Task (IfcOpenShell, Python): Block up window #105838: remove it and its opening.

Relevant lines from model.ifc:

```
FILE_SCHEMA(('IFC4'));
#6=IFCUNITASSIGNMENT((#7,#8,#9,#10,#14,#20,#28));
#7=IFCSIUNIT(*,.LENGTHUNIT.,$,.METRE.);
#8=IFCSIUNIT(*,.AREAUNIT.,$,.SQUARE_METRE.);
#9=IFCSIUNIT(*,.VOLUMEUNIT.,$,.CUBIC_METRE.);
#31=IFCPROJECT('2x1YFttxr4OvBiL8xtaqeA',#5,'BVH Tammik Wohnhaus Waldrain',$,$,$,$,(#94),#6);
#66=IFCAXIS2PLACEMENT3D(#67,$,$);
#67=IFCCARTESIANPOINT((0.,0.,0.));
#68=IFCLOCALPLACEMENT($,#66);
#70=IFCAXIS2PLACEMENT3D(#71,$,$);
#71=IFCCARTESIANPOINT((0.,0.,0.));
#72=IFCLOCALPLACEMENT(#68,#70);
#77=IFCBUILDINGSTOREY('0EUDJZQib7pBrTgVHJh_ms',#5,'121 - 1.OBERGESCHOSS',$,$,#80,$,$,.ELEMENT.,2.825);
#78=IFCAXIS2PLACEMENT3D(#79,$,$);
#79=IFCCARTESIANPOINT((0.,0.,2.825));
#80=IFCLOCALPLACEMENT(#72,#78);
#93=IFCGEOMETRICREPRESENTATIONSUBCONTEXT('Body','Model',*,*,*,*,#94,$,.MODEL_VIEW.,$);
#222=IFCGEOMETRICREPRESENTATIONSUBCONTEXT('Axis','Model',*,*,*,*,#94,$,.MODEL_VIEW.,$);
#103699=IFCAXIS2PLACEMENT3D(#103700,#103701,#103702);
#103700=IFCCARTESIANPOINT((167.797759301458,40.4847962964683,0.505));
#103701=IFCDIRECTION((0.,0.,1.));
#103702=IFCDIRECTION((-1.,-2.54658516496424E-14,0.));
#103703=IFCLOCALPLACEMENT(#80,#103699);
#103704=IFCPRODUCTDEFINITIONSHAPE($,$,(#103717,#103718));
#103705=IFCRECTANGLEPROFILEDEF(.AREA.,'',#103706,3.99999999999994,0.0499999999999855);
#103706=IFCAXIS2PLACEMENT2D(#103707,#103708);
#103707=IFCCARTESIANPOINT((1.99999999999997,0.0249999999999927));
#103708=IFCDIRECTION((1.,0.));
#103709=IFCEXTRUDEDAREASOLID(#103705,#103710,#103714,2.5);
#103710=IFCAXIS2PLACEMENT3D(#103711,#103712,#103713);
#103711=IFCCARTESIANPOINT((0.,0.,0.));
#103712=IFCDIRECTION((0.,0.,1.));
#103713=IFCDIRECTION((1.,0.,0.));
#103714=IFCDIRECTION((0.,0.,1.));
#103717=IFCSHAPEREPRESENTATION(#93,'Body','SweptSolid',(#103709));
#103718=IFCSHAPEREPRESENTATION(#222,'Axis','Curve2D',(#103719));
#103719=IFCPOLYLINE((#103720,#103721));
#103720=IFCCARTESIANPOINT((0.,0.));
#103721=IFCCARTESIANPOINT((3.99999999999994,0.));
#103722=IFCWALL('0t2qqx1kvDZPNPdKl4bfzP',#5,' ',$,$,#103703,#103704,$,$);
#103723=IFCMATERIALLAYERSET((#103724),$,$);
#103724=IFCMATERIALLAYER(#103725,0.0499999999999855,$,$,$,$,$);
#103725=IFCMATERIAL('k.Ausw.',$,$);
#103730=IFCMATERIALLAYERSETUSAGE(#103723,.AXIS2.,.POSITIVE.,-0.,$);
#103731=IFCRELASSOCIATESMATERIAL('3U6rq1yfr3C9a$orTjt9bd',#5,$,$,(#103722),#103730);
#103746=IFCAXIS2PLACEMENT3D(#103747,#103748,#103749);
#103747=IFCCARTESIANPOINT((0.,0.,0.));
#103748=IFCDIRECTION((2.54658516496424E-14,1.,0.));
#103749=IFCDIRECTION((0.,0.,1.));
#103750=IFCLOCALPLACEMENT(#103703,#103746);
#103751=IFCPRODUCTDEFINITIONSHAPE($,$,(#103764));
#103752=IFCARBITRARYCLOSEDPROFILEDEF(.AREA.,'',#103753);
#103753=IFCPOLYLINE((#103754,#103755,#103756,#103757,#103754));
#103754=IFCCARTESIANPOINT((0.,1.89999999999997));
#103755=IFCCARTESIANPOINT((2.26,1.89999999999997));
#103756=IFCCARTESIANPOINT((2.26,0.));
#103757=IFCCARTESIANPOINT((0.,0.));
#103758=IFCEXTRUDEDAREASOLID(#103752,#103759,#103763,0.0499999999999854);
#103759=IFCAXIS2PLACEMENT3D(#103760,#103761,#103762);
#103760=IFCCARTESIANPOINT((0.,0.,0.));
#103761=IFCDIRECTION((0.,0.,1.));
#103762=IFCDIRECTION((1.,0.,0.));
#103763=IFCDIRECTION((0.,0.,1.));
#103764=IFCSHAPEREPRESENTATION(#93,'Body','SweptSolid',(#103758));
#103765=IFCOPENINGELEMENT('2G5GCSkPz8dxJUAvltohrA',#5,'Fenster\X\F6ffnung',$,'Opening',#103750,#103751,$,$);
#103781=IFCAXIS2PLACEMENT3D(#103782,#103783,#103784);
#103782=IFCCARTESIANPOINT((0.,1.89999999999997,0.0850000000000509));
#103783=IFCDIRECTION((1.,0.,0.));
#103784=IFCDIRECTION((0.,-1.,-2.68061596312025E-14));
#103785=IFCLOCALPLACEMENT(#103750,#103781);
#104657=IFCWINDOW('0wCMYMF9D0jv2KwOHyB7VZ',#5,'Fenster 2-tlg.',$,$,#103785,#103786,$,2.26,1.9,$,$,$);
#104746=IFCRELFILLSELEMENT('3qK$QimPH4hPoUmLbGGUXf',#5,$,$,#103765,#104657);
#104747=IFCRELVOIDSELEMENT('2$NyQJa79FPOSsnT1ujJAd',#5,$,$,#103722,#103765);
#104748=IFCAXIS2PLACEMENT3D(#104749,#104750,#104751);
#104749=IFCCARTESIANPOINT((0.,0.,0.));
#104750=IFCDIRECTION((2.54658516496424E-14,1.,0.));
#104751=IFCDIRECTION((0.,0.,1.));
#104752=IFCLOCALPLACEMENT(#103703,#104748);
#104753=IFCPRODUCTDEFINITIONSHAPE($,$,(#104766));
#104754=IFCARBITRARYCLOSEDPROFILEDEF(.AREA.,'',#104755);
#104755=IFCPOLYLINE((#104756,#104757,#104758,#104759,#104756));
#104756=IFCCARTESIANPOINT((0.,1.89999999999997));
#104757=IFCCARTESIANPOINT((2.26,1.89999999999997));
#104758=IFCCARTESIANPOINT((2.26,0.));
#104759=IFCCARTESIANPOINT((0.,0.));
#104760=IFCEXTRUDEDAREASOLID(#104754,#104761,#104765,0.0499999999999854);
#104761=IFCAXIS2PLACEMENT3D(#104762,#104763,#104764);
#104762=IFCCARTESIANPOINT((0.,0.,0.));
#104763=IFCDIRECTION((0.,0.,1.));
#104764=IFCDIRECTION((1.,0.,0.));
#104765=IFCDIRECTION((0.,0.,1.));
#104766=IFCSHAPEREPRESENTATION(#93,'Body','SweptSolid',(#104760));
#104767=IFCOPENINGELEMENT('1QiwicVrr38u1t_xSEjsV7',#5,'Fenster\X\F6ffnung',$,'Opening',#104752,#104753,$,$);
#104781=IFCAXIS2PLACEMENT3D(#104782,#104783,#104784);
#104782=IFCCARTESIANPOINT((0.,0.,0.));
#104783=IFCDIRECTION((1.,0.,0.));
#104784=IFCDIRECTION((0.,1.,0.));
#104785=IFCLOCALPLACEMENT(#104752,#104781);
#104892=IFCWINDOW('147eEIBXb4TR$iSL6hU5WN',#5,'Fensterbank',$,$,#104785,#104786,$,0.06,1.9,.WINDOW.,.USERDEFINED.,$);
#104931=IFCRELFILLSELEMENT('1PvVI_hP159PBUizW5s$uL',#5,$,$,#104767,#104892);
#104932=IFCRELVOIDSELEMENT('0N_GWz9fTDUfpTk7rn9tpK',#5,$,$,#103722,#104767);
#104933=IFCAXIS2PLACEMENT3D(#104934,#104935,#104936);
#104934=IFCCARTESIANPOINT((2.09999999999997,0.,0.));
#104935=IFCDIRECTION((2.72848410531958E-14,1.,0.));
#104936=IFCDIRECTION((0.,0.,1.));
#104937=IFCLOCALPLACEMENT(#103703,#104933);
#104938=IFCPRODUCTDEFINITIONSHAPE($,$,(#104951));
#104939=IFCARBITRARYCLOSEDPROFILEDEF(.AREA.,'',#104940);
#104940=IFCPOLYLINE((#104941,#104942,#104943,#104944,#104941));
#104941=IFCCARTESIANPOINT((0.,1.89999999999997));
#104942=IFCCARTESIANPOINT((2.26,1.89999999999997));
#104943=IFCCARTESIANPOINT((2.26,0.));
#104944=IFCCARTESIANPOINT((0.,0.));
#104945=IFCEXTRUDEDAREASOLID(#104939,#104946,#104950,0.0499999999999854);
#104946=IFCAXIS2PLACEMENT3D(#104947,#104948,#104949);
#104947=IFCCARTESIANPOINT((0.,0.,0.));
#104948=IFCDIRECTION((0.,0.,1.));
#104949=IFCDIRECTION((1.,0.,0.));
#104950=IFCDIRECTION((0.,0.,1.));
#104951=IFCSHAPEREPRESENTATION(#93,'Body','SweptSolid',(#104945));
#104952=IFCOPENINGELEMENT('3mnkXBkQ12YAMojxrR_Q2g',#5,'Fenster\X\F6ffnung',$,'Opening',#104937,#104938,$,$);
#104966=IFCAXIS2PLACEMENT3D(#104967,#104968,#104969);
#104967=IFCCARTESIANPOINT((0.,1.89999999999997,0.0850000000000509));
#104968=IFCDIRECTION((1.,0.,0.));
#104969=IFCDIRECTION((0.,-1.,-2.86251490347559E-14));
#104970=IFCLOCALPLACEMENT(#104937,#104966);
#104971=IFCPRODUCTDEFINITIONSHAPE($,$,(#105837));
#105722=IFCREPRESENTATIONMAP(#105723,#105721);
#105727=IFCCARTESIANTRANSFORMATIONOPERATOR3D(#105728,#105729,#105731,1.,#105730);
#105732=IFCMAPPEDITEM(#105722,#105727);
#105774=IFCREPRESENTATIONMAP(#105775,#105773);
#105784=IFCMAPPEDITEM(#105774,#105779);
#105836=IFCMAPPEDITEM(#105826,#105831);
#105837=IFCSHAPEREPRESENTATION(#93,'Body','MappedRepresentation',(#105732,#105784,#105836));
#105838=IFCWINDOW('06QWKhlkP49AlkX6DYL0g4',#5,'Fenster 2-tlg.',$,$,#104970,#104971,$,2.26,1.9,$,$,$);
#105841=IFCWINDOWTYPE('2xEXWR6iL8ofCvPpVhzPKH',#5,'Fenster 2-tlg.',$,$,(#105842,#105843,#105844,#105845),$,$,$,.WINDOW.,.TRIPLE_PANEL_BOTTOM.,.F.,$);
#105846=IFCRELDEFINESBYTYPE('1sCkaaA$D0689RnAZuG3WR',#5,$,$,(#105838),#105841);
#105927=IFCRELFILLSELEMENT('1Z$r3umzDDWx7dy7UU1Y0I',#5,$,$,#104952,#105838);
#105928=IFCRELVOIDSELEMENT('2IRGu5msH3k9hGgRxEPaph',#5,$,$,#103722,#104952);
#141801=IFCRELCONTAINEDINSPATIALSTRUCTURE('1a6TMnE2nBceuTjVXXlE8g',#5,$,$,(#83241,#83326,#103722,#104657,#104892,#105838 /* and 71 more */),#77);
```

```python
import ifcopenshell
import ifcopenshell.api.feature
import ifcopenshell.api.root
import ifcopenshell.geom
import ifcopenshell.util.shape

model = ifcopenshell.open("model.ifc")
settings = ifcopenshell.geom.settings()


def volume(element):
    """Net volume in cubic metres, openings subtracted."""
    shape = ifcopenshell.geom.create_shape(settings, element)
    return ifcopenshell.util.shape.get_volume(shape.geometry)


window = model.by_id(105838)
opening = window.FillsVoids[0].RelatingOpeningElement
wall = opening.VoidsElements[0].RelatingBuildingElement
before = volume(wall)

ifcopenshell.api.root.remove_product(model, product=window)
ifcopenshell.api.feature.remove_feature(model, feature=opening)

after = volume(wall)

print(f"wall volume {before:.3f} -> {after:.3f} m3")

model.write("model_edited.ifc")
```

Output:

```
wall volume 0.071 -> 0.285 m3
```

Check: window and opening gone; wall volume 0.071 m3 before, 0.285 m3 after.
